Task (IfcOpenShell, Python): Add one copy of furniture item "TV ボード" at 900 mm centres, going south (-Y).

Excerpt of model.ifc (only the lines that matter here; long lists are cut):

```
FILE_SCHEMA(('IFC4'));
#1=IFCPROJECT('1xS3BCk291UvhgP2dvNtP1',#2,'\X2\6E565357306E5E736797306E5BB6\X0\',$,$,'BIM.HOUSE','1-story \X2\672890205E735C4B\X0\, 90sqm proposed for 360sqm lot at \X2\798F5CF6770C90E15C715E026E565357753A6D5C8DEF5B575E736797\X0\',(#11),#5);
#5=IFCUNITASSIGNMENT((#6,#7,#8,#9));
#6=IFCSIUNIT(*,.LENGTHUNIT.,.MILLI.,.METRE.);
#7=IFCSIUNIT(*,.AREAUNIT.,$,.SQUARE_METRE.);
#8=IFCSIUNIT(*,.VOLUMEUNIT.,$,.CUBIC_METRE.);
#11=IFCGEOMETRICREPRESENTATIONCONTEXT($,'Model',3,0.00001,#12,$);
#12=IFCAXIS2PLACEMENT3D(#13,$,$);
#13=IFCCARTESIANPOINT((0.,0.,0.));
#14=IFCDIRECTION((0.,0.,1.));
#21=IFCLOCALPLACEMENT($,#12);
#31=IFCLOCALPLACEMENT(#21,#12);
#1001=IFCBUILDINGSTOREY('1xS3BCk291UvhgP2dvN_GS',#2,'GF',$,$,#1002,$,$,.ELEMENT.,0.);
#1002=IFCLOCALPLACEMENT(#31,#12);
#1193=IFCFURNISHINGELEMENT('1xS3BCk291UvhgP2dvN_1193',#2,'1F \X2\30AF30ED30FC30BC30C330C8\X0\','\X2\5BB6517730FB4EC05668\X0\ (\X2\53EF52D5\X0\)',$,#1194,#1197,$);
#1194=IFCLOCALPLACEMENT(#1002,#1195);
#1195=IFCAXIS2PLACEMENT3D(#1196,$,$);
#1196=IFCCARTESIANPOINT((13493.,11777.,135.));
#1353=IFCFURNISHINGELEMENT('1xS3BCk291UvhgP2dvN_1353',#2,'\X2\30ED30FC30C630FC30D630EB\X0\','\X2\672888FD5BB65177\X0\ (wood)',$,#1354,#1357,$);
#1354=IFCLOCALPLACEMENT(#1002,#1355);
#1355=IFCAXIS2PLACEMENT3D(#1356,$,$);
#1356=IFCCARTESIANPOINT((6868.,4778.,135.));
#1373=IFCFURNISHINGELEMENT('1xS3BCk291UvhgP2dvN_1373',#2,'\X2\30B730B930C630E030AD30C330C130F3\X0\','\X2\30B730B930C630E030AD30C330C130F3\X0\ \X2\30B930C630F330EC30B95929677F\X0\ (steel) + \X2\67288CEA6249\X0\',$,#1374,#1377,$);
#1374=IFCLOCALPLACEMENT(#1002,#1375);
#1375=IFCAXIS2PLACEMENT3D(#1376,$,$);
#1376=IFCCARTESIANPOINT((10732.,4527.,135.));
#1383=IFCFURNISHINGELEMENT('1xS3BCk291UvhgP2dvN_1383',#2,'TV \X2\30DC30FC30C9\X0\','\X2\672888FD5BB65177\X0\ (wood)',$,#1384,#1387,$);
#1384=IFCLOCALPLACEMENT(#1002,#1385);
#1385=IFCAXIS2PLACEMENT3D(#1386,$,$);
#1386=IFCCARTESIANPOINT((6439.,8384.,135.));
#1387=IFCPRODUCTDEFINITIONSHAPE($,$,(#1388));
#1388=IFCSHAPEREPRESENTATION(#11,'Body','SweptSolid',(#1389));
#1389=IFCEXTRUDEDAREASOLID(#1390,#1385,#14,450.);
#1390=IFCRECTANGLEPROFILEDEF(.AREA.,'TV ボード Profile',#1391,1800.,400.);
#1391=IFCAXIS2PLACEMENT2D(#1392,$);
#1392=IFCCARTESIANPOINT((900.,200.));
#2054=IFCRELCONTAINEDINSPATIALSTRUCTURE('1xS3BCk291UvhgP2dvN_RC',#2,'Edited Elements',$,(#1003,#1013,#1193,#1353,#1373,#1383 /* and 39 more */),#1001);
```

```python
import numpy as np
import ifcopenshell
import ifcopenshell.api.geometry
import ifcopenshell.api.root
import ifcopenshell.util.element
import ifcopenshell.util.placement

model = ifcopenshell.open("model.ifc")


def reuse_history(source, copy):
    """copy_class also copies each property set's owner history, people and application; keep the originals."""
    for rel in copy.IsDefinedBy:
        if rel.is_a("IfcRelDefinesByProperties") and (history := rel.RelatingPropertyDefinition.OwnerHistory):
            rel.RelatingPropertyDefinition.OwnerHistory = source.OwnerHistory
            ifcopenshell.util.element.remove_deep2(model, history)


source = model.by_id(1383)
base = ifcopenshell.util.placement.get_local_placement(source.ObjectPlacement)
step = np.array([0.0, -1.0, 0.0]) * 900.0

for i in range(1, 2):
    copy = ifcopenshell.api.root.copy_class(model, product=source)
    copy.Representation = ifcopenshell.util.element.copy_deep(
        model, source.Representation, exclude=["IfcGeometricRepresentationContext", "IfcRepresentationMap"]
    )
    reuse_history(source, copy)
    matrix = base.copy()
    matrix[:3, 3] += i * step
    print("added at", matrix[:3, 3].round(3) + 0.0)
    ifcopenshell.api.geometry.edit_object_placement(model, product=copy, matrix=matrix, is_si=False)

model.write("model_rev.ifc")
```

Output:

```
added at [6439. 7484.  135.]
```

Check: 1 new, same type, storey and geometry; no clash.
